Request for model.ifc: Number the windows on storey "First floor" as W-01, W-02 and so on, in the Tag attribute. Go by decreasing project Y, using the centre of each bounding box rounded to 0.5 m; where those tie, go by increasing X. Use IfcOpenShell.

First a look at what the model holds.

```python
import ifcopenshell
import ifcopenshell.util.element
import ifcopenshell.util.placement

model = ifcopenshell.open("model.ifc")
print(model.schema)
storey = next(s for s in model.by_type("IfcBuildingStorey") if s.Name == "First floor")
windows = [e for e in ifcopenshell.util.element.get_decomposition(storey) if e.is_a("IfcWindow")]
for e in sorted(windows, key=lambda e: e.id()):
    origin = ifcopenshell.util.placement.get_local_placement(e.ObjectPlacement)[:3, 3]
    print(e.id(), e.Tag, e.Name, origin.round(2) + 0.0, sep=" | ")
```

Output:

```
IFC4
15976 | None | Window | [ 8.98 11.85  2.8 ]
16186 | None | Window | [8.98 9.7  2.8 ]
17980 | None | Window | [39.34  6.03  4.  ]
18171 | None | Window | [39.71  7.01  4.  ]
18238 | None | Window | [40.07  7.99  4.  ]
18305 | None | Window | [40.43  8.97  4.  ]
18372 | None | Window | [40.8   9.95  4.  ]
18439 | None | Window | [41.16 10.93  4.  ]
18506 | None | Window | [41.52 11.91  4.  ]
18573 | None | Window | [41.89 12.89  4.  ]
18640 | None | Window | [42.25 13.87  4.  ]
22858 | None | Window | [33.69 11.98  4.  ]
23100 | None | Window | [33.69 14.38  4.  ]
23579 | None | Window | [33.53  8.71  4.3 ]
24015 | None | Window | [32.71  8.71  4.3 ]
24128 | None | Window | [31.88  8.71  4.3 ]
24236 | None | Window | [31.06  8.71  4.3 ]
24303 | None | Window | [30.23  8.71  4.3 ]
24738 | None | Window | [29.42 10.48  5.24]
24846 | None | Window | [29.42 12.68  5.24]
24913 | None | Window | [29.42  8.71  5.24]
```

```python
import ifcopenshell
import ifcopenshell.geom
import ifcopenshell.util.element
import ifcopenshell.util.shape

model = ifcopenshell.open("model.ifc")
settings = ifcopenshell.geom.settings()
settings.set("use-world-coords", True)


def centre(element):
    shape = ifcopenshell.geom.create_shape(settings, element)
    return ifcopenshell.util.shape.get_bbox_centroid(shape.geometry)


storey = next(s for s in model.by_type("IfcBuildingStorey") if s.Name == "First floor")
windows = [e for e in ifcopenshell.util.element.get_decomposition(storey) if e.is_a("IfcWindow")]

# Insertion points can sit at a corner or the storey origin, so sort by the geometry (in metres).
centres = {e: centre(e) for e in windows}
windows.sort(key=lambda e: (-round(centres[e][1] / 0.5), centres[e][0]))

for i, e in enumerate(windows, start=1):
    number = f"W-{i:02d}"
    e.Tag = number
    print(e.id(), number)

model.write("model_edited.ifc")
```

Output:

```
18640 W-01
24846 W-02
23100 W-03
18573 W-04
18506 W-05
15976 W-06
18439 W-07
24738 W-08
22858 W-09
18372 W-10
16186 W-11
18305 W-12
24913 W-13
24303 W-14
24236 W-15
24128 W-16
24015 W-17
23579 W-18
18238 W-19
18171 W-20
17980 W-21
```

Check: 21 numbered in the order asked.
